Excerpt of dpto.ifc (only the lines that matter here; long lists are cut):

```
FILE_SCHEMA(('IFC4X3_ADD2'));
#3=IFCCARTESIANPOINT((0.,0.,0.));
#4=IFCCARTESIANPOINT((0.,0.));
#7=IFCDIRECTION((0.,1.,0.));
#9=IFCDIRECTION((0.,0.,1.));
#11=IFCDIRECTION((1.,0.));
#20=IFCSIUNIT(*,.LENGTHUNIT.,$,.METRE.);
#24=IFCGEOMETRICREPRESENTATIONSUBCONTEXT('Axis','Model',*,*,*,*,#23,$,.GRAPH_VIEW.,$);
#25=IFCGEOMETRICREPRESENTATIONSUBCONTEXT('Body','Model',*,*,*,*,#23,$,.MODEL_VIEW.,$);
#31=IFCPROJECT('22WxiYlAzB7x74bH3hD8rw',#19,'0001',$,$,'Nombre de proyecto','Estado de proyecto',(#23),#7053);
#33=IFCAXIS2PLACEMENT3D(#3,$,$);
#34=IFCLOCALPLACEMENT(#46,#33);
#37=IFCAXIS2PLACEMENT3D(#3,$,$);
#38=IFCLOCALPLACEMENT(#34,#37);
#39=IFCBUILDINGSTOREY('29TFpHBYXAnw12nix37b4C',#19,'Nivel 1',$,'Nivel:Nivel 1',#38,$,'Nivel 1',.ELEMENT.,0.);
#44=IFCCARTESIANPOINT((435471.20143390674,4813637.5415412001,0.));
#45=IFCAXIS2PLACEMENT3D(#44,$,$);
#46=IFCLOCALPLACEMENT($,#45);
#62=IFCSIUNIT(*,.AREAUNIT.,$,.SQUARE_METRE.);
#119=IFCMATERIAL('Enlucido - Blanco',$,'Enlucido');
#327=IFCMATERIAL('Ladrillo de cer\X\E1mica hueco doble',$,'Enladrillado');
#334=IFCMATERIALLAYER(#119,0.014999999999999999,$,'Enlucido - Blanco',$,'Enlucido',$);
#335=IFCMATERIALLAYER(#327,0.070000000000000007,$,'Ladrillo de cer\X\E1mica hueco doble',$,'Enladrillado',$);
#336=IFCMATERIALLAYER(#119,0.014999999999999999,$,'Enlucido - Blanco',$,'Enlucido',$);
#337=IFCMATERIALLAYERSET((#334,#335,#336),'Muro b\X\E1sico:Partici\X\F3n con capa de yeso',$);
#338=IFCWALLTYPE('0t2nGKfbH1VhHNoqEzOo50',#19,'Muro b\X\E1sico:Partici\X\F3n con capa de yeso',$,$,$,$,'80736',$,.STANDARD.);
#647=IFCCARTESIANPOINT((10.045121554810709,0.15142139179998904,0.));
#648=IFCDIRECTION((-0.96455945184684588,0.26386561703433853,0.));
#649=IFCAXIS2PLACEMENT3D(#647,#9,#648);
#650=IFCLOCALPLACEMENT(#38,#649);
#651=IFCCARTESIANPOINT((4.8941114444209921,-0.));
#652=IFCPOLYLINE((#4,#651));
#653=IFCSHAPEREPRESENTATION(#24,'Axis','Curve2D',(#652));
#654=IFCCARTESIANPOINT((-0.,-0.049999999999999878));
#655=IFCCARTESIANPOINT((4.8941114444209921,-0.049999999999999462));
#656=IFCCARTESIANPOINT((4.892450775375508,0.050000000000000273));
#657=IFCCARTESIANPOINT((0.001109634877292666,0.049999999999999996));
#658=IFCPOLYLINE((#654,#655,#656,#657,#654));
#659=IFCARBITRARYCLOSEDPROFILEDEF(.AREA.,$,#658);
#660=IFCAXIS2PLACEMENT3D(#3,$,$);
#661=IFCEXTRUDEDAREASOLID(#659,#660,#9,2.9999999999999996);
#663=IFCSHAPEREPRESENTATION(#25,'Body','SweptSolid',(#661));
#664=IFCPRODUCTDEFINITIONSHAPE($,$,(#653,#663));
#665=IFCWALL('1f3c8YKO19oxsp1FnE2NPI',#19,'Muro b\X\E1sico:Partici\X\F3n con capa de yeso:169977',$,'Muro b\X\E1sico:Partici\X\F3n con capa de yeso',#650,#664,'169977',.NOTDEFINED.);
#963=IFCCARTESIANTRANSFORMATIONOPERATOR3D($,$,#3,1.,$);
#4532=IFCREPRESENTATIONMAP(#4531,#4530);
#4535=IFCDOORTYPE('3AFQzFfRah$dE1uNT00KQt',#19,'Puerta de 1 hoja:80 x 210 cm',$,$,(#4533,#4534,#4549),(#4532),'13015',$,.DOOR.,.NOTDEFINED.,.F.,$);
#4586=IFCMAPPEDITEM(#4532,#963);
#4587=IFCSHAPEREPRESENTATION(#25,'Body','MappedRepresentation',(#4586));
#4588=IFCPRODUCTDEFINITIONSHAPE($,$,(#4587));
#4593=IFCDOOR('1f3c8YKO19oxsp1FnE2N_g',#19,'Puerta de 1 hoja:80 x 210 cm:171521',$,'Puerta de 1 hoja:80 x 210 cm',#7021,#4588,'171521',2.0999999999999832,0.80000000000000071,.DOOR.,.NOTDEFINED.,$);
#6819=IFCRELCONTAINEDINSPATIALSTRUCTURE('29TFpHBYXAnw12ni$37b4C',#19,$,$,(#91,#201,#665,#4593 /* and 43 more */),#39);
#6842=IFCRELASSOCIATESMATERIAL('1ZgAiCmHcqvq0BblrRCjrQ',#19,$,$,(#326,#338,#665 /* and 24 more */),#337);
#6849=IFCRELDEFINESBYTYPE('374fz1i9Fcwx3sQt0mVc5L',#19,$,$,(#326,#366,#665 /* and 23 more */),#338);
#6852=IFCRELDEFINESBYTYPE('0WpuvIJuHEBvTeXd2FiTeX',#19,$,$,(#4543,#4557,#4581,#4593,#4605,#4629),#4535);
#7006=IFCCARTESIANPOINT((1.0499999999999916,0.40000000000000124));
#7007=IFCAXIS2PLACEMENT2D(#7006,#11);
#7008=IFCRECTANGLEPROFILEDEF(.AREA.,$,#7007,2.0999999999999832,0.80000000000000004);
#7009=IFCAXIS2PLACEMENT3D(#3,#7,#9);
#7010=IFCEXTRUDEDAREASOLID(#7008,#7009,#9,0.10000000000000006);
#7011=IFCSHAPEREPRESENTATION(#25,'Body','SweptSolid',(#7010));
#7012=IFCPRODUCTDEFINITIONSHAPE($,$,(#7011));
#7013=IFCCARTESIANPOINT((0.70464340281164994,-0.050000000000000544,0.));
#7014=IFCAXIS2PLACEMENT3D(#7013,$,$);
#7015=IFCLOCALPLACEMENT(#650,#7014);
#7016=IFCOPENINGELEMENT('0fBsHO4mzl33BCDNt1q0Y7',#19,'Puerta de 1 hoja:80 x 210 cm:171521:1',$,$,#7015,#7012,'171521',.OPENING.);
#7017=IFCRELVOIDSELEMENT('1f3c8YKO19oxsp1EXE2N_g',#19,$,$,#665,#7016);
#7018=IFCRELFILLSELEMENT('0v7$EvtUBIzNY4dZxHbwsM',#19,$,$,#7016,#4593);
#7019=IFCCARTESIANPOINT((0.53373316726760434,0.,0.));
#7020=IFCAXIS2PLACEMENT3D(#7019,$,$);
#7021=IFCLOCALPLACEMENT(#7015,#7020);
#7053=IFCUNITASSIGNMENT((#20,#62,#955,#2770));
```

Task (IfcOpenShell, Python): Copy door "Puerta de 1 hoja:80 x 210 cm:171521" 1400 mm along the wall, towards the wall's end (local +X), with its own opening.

```python
import ifcopenshell
import ifcopenshell.api.feature
import ifcopenshell.api.geometry
import ifcopenshell.api.root
import ifcopenshell.geom
import ifcopenshell.util.element
import ifcopenshell.util.placement
import ifcopenshell.util.shape
import ifcopenshell.util.unit

model = ifcopenshell.open("dpto.ifc")
unit_scale = ifcopenshell.util.unit.calculate_unit_scale(model)
settings = ifcopenshell.geom.settings()


def volume(element):
    """Net volume in cubic metres, openings subtracted."""
    shape = ifcopenshell.geom.create_shape(settings, element)
    return ifcopenshell.util.shape.get_volume(shape.geometry)


def reuse_history(source, copy):
    """copy_class also copies each property set's owner history, people and application; keep the originals."""
    for rel in copy.IsDefinedBy:
        if rel.is_a("IfcRelDefinesByProperties") and (history := rel.RelatingPropertyDefinition.OwnerHistory):
            rel.RelatingPropertyDefinition.OwnerHistory = source.OwnerHistory
            ifcopenshell.util.element.remove_deep2(model, history)


door = model.by_id(4593)
opening = door.FillsVoids[0].RelatingOpeningElement
wall = opening.VoidsElements[0].RelatingBuildingElement
before = volume(wall)
shift = ifcopenshell.util.placement.get_local_placement(wall.ObjectPlacement)[:3, 0] * 1.4 / unit_scale

# copy_class copies the void relationship, type, container and properties, but no geometry.
new_opening = ifcopenshell.api.root.copy_class(model, product=opening)
new_opening.Representation = ifcopenshell.util.element.copy_deep(
    model, opening.Representation, exclude=["IfcGeometricRepresentationContext", "IfcRepresentationMap"]
)
new_opening.Name = "Puerta de 1 hoja:80 x 210 cm"
new_opening.Tag = None
new_door = ifcopenshell.api.root.copy_class(model, product=door)
new_door.Representation = ifcopenshell.util.element.copy_deep(
    model, door.Representation, exclude=["IfcGeometricRepresentationContext", "IfcRepresentationMap"]
)
new_door.Name = "Puerta de 1 hoja:80 x 210 cm"
new_door.Tag = None
reuse_history(door, new_door)
ifcopenshell.api.feature.add_filling(model, opening=new_opening, element=new_door)

for old, new in ((opening, new_opening), (door, new_door)):
    matrix = ifcopenshell.util.placement.get_local_placement(old.ObjectPlacement)
    matrix[:3, 3] += shift
    ifcopenshell.api.geometry.edit_object_placement(model, product=new, matrix=matrix, is_si=False)

after = volume(wall)

print(f"wall volume {before:.3f} -> {after:.3f} m3")

model.write("dpto_edited.ifc")
```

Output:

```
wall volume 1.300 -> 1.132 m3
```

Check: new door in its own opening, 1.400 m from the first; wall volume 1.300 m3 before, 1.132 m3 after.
